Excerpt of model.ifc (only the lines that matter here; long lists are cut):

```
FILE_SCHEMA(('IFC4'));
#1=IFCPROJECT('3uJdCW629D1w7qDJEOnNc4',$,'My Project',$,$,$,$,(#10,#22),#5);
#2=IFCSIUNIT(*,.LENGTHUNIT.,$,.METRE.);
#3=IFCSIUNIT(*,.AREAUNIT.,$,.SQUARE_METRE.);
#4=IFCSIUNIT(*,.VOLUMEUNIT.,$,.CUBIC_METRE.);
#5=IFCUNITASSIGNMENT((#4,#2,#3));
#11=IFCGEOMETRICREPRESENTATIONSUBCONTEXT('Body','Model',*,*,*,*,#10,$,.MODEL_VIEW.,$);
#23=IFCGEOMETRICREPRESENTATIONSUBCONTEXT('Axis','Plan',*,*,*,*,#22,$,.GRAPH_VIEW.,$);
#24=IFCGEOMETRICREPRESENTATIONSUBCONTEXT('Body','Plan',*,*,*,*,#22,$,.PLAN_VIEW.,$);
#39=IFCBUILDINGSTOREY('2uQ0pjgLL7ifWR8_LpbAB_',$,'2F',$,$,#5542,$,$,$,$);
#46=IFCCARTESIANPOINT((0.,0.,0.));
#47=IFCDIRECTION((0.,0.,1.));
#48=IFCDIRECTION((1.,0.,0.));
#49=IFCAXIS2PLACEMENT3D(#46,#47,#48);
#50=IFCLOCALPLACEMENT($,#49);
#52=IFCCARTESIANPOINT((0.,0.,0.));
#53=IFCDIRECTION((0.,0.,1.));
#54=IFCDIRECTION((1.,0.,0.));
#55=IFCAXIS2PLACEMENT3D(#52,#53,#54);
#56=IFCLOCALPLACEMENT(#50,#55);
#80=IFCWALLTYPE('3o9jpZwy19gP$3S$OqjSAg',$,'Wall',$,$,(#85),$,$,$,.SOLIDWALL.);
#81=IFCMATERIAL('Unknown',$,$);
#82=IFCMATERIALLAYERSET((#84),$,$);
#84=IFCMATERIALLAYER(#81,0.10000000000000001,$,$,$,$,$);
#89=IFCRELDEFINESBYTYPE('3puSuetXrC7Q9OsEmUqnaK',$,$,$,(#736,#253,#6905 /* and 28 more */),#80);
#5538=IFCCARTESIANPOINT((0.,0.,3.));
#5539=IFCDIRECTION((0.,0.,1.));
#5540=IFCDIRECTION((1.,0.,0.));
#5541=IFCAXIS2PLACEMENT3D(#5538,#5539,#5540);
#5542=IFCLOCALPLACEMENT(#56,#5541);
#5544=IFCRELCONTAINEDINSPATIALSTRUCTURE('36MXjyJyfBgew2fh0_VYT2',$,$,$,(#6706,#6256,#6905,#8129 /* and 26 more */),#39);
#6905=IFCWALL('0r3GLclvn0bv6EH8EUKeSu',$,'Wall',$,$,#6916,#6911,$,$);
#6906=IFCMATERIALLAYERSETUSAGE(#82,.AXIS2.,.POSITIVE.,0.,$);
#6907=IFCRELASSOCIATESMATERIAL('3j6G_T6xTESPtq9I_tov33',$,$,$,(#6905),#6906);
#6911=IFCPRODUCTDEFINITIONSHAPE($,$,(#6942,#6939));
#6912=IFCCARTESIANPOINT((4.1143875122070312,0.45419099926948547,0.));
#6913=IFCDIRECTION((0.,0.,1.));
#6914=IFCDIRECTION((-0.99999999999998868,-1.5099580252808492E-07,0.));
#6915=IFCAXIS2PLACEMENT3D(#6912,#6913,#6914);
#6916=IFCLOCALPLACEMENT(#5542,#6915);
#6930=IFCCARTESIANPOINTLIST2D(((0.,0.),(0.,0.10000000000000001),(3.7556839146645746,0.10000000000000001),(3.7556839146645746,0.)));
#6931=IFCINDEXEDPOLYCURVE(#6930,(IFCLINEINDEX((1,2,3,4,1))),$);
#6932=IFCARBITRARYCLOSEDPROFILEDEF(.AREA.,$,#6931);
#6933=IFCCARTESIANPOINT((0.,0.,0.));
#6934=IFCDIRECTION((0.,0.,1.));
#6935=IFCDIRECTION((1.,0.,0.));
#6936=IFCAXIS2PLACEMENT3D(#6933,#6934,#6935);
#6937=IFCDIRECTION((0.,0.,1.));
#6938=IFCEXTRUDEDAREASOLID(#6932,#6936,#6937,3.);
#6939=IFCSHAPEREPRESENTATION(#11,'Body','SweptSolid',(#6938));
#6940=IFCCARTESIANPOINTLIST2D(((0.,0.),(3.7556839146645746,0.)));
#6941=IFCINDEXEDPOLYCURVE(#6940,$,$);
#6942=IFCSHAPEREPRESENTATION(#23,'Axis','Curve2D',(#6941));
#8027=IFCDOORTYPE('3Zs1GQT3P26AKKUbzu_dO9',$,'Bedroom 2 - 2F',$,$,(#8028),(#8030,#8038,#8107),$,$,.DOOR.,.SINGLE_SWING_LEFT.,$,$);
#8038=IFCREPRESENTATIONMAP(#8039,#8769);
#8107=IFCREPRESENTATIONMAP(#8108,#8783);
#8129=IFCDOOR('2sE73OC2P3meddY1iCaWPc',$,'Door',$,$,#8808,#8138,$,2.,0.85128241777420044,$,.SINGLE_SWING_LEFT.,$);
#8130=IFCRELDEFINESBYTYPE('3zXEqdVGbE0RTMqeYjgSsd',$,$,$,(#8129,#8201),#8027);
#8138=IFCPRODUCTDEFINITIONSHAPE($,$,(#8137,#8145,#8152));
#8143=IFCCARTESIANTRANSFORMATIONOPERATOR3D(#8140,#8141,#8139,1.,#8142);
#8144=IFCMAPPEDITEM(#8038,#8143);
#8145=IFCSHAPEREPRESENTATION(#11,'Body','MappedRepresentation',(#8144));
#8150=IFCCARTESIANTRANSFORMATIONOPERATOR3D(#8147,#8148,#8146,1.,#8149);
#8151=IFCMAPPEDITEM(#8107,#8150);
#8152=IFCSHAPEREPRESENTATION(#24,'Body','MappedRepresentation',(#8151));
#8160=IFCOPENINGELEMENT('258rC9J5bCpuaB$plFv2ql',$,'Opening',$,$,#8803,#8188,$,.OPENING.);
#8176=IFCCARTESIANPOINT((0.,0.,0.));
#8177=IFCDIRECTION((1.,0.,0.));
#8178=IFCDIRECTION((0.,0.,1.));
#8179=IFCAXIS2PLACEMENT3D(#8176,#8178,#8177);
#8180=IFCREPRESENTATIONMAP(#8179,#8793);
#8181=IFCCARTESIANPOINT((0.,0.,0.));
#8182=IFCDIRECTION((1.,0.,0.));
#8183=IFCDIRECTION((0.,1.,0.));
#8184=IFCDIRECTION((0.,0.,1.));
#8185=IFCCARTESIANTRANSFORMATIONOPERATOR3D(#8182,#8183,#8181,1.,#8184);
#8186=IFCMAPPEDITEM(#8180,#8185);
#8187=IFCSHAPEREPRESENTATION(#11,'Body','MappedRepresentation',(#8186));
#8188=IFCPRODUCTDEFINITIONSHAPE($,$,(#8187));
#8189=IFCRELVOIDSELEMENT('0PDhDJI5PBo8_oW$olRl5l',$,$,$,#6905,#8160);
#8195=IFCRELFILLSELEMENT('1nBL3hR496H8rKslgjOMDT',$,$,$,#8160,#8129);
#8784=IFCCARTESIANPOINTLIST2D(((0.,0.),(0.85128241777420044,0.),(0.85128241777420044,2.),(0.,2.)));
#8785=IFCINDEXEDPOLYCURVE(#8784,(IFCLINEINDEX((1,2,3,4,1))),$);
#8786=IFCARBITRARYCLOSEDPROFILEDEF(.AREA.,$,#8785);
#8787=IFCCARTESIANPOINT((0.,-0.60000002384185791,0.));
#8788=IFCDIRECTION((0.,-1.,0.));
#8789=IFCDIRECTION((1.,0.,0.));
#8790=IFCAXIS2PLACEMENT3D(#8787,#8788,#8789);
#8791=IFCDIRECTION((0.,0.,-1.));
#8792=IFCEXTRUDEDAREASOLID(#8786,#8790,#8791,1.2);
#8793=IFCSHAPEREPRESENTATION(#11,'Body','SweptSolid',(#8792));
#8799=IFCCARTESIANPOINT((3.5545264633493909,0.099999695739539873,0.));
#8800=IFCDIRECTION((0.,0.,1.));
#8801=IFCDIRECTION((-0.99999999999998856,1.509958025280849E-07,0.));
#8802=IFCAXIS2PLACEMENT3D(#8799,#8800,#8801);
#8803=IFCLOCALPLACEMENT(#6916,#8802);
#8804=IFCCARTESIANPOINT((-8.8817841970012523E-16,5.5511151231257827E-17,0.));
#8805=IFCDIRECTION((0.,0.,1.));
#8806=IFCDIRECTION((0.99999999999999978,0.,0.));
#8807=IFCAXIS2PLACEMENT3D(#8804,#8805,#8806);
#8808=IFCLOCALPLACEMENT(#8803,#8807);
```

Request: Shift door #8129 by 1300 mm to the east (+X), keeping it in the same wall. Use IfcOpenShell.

```python
import ifcopenshell
import ifcopenshell.api.geometry
import ifcopenshell.util.placement
import ifcopenshell.util.unit

model = ifcopenshell.open("model.ifc")
unit_scale = ifcopenshell.util.unit.calculate_unit_scale(model)

door = model.by_guid("2sE73OC2P3meddY1iCaWPc")
opening = door.FillsVoids[0].RelatingOpeningElement
wall = opening.VoidsElements[0].RelatingBuildingElement

wall_matrix = ifcopenshell.util.placement.get_local_placement(wall.ObjectPlacement)
shift = wall_matrix[:3, 0] * -1.3 / unit_scale
before = ifcopenshell.util.placement.get_local_placement(door.ObjectPlacement)[:3, 3].copy()

# The door is placed relative to its opening, so it follows when the opening moves.
matrix = ifcopenshell.util.placement.get_local_placement(opening.ObjectPlacement)
matrix[:3, 3] += shift
ifcopenshell.api.geometry.edit_object_placement(
    model, product=opening, matrix=matrix, is_si=False, should_transform_children=True
)

after = ifcopenshell.util.placement.get_local_placement(door.ObjectPlacement)[:3, 3]
print("door moved by", (after - before).round(3) + 0.0)

model.write("model_rev.ifc")
```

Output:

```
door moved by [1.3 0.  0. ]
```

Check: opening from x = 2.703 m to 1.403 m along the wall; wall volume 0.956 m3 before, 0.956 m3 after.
